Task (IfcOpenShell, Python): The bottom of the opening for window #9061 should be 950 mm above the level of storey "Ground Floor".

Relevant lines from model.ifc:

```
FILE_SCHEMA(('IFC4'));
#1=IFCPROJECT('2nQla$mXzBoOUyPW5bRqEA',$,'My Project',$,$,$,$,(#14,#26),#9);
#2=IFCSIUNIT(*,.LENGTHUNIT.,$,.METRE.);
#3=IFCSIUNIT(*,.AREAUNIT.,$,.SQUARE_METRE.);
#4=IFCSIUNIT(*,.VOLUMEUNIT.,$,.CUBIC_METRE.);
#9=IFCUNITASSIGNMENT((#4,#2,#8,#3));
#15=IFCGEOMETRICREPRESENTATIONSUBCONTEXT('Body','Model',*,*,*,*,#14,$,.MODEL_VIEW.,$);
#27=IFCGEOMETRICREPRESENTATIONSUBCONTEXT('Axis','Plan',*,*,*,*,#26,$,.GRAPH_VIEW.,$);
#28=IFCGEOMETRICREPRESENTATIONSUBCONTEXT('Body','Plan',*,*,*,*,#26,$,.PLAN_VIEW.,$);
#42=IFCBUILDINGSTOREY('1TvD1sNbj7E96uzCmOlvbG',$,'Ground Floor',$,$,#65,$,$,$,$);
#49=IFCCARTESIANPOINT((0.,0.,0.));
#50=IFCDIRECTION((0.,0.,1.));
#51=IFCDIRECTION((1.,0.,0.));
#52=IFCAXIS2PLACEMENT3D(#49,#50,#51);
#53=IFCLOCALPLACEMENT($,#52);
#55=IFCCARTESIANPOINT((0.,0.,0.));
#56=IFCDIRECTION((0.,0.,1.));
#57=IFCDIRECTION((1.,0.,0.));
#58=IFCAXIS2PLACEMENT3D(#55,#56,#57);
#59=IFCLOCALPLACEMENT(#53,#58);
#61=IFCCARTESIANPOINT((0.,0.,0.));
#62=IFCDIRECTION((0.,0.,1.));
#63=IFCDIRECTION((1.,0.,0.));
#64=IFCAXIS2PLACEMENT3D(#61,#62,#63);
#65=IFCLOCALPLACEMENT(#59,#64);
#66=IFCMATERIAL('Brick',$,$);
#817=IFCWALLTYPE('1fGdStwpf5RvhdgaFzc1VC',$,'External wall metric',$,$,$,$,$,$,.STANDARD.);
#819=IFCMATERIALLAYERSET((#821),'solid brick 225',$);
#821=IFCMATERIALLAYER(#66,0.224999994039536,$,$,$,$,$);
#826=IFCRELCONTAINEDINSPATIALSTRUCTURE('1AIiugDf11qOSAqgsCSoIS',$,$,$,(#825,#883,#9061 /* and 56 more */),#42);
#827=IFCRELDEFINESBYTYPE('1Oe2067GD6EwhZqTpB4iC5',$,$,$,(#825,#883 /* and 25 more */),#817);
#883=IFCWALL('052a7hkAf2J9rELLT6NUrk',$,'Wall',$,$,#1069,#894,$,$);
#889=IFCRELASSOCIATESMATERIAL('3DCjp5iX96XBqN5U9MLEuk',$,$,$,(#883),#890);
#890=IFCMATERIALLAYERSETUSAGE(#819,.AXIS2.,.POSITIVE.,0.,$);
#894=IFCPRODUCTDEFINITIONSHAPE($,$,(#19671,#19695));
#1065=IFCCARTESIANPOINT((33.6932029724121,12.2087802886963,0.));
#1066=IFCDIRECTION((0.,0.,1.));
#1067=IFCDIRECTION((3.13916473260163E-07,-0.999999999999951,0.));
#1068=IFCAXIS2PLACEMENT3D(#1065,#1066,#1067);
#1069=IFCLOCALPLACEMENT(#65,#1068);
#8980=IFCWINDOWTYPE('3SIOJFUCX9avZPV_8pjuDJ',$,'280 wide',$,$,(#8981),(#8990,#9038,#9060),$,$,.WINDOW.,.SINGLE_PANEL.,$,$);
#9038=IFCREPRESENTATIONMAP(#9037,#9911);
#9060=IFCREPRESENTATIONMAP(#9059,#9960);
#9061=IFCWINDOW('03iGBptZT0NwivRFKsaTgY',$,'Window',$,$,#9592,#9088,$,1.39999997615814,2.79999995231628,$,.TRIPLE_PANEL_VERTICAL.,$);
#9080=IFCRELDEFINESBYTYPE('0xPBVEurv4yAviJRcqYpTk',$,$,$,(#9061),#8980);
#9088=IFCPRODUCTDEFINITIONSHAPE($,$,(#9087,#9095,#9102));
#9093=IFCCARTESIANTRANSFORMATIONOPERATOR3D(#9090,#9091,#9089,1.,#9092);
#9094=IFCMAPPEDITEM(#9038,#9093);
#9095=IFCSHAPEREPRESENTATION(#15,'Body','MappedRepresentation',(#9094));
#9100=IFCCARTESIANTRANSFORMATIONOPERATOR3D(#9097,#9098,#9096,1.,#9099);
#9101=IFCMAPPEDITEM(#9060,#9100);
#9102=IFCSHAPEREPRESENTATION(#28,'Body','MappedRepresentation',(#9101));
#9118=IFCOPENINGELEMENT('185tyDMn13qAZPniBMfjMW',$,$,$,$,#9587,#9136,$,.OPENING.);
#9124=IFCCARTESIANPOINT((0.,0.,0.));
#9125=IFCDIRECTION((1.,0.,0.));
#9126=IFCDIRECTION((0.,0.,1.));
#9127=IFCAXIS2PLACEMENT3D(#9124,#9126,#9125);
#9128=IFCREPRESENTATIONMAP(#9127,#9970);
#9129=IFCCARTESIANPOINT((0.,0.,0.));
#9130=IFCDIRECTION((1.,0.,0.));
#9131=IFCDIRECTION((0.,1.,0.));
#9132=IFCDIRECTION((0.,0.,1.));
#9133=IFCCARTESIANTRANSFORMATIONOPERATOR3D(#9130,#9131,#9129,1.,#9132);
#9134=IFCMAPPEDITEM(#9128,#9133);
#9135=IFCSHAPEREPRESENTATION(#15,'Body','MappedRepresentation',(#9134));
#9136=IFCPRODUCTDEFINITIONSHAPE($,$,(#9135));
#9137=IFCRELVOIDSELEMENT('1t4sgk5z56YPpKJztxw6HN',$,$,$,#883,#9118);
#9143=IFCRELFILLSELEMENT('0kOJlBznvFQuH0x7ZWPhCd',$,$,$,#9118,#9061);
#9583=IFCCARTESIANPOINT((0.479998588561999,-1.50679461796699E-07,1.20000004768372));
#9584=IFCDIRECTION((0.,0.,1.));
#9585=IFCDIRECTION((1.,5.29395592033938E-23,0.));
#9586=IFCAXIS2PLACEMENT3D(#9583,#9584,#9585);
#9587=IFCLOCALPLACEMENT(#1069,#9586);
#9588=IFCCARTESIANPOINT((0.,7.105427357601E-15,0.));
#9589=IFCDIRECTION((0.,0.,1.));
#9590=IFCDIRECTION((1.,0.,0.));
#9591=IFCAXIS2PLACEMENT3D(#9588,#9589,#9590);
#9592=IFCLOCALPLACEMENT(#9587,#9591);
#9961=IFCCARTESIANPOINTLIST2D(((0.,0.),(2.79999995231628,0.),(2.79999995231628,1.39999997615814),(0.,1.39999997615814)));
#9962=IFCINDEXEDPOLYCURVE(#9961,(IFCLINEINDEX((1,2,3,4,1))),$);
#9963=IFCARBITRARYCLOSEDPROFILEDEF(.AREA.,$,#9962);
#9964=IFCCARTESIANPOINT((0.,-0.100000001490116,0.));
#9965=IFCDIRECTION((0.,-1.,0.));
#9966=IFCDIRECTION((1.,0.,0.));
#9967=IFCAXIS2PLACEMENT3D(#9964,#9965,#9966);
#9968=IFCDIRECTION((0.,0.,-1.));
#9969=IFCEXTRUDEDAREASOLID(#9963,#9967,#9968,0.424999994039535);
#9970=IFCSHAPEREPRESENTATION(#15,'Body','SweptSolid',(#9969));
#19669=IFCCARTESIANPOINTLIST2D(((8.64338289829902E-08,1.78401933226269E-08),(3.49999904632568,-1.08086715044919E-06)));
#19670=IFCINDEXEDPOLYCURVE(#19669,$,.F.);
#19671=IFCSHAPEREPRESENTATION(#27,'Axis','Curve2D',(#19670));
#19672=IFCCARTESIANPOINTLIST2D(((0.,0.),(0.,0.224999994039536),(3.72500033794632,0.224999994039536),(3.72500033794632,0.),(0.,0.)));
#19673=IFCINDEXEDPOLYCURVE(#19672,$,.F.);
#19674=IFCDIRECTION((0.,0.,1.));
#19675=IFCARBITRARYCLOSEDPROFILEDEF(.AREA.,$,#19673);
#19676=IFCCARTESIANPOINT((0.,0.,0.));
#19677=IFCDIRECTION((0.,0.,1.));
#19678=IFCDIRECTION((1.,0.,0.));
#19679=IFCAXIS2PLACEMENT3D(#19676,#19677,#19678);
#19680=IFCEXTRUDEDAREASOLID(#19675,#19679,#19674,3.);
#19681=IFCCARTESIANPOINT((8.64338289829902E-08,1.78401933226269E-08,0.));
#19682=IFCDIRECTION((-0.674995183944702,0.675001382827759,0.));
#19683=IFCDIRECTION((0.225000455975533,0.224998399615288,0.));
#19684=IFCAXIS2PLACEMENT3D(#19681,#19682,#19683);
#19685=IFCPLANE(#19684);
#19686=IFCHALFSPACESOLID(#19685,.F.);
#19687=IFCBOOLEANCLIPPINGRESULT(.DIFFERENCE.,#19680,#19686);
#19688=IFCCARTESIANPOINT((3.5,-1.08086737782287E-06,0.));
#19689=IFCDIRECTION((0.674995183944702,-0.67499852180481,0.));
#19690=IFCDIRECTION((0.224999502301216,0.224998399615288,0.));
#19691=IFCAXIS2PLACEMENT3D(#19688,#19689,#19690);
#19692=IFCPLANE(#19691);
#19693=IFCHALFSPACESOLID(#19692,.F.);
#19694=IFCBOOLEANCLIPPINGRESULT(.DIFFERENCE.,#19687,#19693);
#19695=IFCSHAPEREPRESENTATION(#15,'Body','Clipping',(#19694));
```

```python
import numpy as np
import ifcopenshell
import ifcopenshell.api.geometry
import ifcopenshell.geom
import ifcopenshell.util.element
import ifcopenshell.util.placement
import ifcopenshell.util.shape
import ifcopenshell.util.unit

model = ifcopenshell.open("model.ifc")
unit_scale = ifcopenshell.util.unit.calculate_unit_scale(model)

window = model.by_guid("03iGBptZT0NwivRFKsaTgY")
opening = window.FillsVoids[0].RelatingOpeningElement
storey = ifcopenshell.util.element.get_container(window, ifc_class="IfcBuildingStorey")
level = ifcopenshell.util.placement.get_local_placement(storey.ObjectPlacement)[2, 3]

# The opening's origin need not be at the sill, so measure its lowest point.
shape = ifcopenshell.geom.create_shape(ifcopenshell.geom.settings(), opening)
bottom = ifcopenshell.util.shape.get_shape_bottom_elevation(shape, shape.geometry) / unit_scale
dz = level + 0.95 - bottom

shift = np.array([0.0, 0.0, dz])
# The window is placed relative to its opening, so it follows when the opening moves.
matrix = ifcopenshell.util.placement.get_local_placement(opening.ObjectPlacement)
matrix[:3, 3] += shift
ifcopenshell.api.geometry.edit_object_placement(
    model, product=opening, matrix=matrix, is_si=False, should_transform_children=True
)

print(f"moved by {dz * unit_scale:+.3f} m")

model.write("model-out.ifc")
```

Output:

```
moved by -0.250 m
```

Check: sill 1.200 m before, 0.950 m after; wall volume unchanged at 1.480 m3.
